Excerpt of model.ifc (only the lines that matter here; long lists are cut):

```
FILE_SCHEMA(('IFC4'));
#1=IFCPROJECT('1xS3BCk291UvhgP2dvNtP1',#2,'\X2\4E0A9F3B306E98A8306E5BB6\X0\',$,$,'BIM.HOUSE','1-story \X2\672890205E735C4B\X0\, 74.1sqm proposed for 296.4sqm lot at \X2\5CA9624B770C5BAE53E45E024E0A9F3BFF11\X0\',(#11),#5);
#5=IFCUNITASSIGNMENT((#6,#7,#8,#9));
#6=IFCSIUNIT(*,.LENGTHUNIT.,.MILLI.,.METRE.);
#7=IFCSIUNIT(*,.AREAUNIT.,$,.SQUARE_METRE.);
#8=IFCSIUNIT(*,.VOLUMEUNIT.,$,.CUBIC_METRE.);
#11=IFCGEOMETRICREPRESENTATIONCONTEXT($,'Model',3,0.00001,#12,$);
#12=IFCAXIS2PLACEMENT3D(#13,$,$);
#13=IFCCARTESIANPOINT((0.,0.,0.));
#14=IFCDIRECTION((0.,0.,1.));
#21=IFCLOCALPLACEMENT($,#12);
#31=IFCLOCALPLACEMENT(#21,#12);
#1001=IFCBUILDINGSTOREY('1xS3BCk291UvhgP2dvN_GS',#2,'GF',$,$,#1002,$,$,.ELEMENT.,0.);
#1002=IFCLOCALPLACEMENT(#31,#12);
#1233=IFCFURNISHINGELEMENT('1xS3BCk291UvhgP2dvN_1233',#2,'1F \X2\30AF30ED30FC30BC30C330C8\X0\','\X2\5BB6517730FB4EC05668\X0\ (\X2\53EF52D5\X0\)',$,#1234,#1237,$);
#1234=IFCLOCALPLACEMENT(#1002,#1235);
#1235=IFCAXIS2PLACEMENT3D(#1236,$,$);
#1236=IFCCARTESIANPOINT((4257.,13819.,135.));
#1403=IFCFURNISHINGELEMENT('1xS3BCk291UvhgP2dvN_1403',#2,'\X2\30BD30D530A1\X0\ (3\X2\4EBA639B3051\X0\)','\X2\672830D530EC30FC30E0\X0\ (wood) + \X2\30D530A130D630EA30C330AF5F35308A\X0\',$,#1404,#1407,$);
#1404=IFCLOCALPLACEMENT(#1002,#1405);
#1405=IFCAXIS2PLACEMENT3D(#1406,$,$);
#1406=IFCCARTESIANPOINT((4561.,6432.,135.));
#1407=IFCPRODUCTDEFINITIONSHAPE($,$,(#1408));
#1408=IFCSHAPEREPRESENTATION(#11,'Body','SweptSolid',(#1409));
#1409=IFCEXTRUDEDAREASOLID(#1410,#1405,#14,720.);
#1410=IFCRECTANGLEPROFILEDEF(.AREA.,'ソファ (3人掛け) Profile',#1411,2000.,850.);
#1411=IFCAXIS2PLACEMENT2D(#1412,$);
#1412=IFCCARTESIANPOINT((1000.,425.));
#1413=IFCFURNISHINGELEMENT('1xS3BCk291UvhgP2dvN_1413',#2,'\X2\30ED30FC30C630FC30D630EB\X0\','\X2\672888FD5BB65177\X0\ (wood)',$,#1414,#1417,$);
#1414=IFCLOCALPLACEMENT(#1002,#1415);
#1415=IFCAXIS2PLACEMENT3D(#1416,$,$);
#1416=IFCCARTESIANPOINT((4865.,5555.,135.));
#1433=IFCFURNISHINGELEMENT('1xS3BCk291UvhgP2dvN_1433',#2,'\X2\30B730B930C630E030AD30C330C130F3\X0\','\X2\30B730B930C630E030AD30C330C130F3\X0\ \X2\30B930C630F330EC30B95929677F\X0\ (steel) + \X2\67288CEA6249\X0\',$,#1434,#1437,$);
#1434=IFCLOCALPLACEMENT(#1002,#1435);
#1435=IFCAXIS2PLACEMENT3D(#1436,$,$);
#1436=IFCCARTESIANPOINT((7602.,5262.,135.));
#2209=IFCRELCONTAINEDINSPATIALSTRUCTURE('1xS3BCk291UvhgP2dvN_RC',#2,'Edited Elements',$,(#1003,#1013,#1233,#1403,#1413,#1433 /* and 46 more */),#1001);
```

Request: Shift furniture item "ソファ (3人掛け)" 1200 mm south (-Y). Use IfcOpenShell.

```python
import ifcopenshell
import ifcopenshell.api.geometry
import ifcopenshell.util.placement

model = ifcopenshell.open("model.ifc")

item = model.by_id(1403)
matrix = ifcopenshell.util.placement.get_local_placement(item.ObjectPlacement)
matrix[1, 3] -= 1200.0
ifcopenshell.api.geometry.edit_object_placement(model, product=item, matrix=matrix, is_si=False)

print(ifcopenshell.util.placement.get_local_placement(item.ObjectPlacement).round(3) + 0.0)

model.write("model_edited.ifc")
```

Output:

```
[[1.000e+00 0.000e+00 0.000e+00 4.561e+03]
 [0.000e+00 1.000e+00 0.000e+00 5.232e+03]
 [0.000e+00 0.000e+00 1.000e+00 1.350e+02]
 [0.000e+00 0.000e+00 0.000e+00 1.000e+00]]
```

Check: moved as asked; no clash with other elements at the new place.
